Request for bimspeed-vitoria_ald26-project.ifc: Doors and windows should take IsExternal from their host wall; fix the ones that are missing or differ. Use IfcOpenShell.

First a look at what the model holds.

```python
import ifcopenshell
import ifcopenshell.util.element

model = ifcopenshell.open("bimspeed-vitoria_ald26-project.ifc")
print(model.schema)
seen = {}
for e in model.by_type("IfcDoor") + model.by_type("IfcWindow"):
    if not e.FillsVoids:
        continue
    host = e.FillsVoids[0].RelatingOpeningElement.VoidsElements[0].RelatingBuildingElement
    own = ifcopenshell.util.element.get_pset(e, f"Pset_{e.is_a()[3:].removesuffix('StandardCase')}Common", "IsExternal")
    wall = ifcopenshell.util.element.get_pset(host, "Pset_WallCommon", "IsExternal")
    seen[e.is_a(), own, wall] = seen.get((e.is_a(), own, wall), 0) + 1
for (cls, own, wall), count in sorted(seen.items(), key=str):
    print(count, cls, "IsExternal:", own, "| host wall:", wall)
```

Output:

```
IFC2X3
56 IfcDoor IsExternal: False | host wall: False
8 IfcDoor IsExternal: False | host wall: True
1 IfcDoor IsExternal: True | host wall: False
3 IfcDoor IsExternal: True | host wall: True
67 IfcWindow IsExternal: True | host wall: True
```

```python
import ifcopenshell
import ifcopenshell.api.pset
import ifcopenshell.util.element

model = ifcopenshell.open("bimspeed-vitoria_ald26-project.ifc")

count = 0
for ifc_class, pset_name in (("IfcDoor", "Pset_DoorCommon"), ("IfcWindow", "Pset_WindowCommon")):
    for e in model.by_type(ifc_class):
        if not e.FillsVoids:
            continue
        host = e.FillsVoids[0].RelatingOpeningElement.VoidsElements[0].RelatingBuildingElement
        external = ifcopenshell.util.element.get_pset(host, "Pset_WallCommon", "IsExternal")
        if external is None or ifcopenshell.util.element.get_pset(e, pset_name, "IsExternal") == external:
            continue
        pset = ifcopenshell.api.pset.add_pset(model, product=e, name=pset_name)
        ifcopenshell.api.pset.edit_pset(model, pset=pset, properties={"IsExternal": external})
        count += 1

print(count, "updated")

model.write("bimspeed-vitoria_ald26-project_updated.ifc")
```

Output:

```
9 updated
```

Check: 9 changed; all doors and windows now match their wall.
